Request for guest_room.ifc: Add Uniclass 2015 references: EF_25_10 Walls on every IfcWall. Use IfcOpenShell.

First a look at what the model holds.

```python
import ifcopenshell

model = ifcopenshell.open("guest_room.ifc")
print(model.schema)
print("classifications:", [c.Name for c in model.by_type("IfcClassification")])
for ifc_class in ("IfcDoor", "IfcRoof", "IfcStair", "IfcWall", "IfcWindow"):
    print(ifc_class, len(model.by_type(ifc_class)))
```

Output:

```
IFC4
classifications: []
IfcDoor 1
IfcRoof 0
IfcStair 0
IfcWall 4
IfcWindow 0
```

```python
import ifcopenshell
import ifcopenshell.api.classification

model = ifcopenshell.open("guest_room.ifc")

system = ifcopenshell.api.classification.add_classification(model, classification="Uniclass 2015")

codes = {
    "IfcWall": ("EF_25_10", "Walls"),
}
for ifc_class, (code, name) in codes.items():
    products = model.by_type(ifc_class)
    ifcopenshell.api.classification.add_reference(
        model, products=products, classification=system, identification=code, name=name
    )
    print(code, len(products))

model.write("guest_room_edited.ifc")
```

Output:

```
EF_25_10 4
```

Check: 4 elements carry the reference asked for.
